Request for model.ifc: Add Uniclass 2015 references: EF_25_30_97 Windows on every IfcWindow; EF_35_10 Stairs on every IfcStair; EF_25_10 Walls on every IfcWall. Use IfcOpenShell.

First a look at what the model holds.

```python
import ifcopenshell

model = ifcopenshell.open("model.ifc")
print(model.schema)
print("classifications:", [c.Name for c in model.by_type("IfcClassification")])
for ifc_class in ("IfcDoor", "IfcRoof", "IfcStair", "IfcWall", "IfcWindow"):
    print(ifc_class, len(model.by_type(ifc_class)))
```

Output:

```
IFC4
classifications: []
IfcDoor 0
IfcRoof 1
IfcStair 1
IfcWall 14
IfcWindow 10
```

```python
import ifcopenshell
import ifcopenshell.api.classification

model = ifcopenshell.open("model.ifc")

system = ifcopenshell.api.classification.add_classification(model, classification="Uniclass 2015")

codes = {
    "IfcWindow": ("EF_25_30_97", "Windows"),
    "IfcStair": ("EF_35_10", "Stairs"),
    "IfcWall": ("EF_25_10", "Walls"),
}
for ifc_class, (code, name) in codes.items():
    products = model.by_type(ifc_class)
    ifcopenshell.api.classification.add_reference(
        model, products=products, classification=system, identification=code, name=name
    )
    print(code, len(products))

model.write("model_updated.ifc")
```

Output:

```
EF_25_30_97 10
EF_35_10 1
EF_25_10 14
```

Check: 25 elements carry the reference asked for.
